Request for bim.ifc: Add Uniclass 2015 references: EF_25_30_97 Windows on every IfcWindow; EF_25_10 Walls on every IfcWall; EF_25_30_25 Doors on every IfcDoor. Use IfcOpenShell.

First a look at what the model holds.

```python
import ifcopenshell

model = ifcopenshell.open("bim.ifc")
print(model.schema)
print("classifications:", [c.Name for c in model.by_type("IfcClassification")])
for ifc_class in ("IfcDoor", "IfcRoof", "IfcStair", "IfcWall", "IfcWindow"):
    print(ifc_class, len(model.by_type(ifc_class)))
```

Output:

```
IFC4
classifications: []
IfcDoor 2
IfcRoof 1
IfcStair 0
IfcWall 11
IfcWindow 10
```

```python
import ifcopenshell
import ifcopenshell.api.classification

model = ifcopenshell.open("bim.ifc")

system = ifcopenshell.api.classification.add_classification(model, classification="Uniclass 2015")

codes = {
    "IfcWindow": ("EF_25_30_97", "Windows"),
    "IfcWall": ("EF_25_10", "Walls"),
    "IfcDoor": ("EF_25_30_25", "Doors"),
}
for ifc_class, (code, name) in codes.items():
    products = model.by_type(ifc_class)
    ifcopenshell.api.classification.add_reference(
        model, products=products, classification=system, identification=code, name=name
    )
    print(code, len(products))

model.write("bim_rev.ifc")
```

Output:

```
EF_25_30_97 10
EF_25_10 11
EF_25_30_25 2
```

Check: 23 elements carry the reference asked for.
